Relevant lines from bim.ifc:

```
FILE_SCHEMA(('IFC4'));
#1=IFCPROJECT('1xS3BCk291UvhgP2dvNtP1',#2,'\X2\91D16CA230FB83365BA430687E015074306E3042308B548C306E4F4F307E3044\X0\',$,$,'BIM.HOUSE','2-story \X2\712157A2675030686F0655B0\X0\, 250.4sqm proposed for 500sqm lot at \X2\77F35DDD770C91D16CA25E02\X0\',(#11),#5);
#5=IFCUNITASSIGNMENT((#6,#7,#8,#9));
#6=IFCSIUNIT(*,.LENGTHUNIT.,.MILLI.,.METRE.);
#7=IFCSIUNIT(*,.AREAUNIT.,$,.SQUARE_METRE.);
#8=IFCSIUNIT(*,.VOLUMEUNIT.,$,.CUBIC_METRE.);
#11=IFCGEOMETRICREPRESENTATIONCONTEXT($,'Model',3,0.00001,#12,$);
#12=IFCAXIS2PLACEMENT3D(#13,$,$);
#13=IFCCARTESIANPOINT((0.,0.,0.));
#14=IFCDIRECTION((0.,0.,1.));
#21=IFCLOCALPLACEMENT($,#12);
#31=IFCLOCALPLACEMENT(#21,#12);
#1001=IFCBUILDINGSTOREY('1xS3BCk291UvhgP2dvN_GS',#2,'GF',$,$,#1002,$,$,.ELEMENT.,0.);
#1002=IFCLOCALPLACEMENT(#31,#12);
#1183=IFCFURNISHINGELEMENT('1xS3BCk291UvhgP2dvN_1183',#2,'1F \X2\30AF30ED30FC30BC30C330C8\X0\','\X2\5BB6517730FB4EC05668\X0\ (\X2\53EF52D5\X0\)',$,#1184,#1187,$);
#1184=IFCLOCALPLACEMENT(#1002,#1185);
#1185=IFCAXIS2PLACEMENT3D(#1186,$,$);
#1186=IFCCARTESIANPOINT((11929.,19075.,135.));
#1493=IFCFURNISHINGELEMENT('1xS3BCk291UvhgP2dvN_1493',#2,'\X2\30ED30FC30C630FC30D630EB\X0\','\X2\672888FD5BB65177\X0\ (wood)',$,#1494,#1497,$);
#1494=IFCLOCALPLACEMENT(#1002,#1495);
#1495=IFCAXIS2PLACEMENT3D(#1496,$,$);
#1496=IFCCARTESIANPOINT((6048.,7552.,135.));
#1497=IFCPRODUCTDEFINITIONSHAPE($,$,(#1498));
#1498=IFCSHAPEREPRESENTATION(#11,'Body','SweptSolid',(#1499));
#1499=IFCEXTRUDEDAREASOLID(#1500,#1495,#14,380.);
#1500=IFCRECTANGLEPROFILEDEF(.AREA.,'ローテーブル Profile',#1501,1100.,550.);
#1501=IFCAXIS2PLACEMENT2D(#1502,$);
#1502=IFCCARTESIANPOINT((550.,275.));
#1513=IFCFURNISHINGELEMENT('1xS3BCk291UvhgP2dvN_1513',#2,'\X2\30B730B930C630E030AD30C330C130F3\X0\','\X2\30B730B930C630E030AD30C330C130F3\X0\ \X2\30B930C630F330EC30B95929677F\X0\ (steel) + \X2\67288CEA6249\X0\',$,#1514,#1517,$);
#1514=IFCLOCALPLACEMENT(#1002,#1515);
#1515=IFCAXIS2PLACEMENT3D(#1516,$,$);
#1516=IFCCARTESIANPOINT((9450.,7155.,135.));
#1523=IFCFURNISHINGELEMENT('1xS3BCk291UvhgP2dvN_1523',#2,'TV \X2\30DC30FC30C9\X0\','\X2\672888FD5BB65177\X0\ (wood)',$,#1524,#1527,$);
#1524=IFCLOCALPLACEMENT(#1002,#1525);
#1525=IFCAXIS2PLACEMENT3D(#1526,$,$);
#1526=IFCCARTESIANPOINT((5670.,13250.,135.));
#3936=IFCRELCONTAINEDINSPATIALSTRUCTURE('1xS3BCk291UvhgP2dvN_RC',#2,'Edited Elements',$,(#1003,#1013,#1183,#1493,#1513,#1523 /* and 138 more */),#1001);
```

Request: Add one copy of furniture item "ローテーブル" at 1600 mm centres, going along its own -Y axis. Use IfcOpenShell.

```python
import ifcopenshell
import ifcopenshell.api.geometry
import ifcopenshell.api.root
import ifcopenshell.util.element
import ifcopenshell.util.placement

model = ifcopenshell.open("bim.ifc")


def reuse_history(source, copy):
    """copy_class also copies each property set's owner history, people and application; keep the originals."""
    for rel in copy.IsDefinedBy:
        if rel.is_a("IfcRelDefinesByProperties") and (history := rel.RelatingPropertyDefinition.OwnerHistory):
            rel.RelatingPropertyDefinition.OwnerHistory = source.OwnerHistory
            ifcopenshell.util.element.remove_deep2(model, history)


source = model.by_id(1493)
base = ifcopenshell.util.placement.get_local_placement(source.ObjectPlacement)
step = -base[:3, 1] * 1600.0

for i in range(1, 2):
    copy = ifcopenshell.api.root.copy_class(model, product=source)
    copy.Representation = ifcopenshell.util.element.copy_deep(
        model, source.Representation, exclude=["IfcGeometricRepresentationContext", "IfcRepresentationMap"]
    )
    reuse_history(source, copy)
    matrix = base.copy()
    matrix[:3, 3] += i * step
    print("added at", matrix[:3, 3].round(3) + 0.0)
    ifcopenshell.api.geometry.edit_object_placement(model, product=copy, matrix=matrix, is_si=False)

model.write("bim_rev.ifc")
```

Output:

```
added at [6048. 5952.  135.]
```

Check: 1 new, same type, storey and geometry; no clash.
